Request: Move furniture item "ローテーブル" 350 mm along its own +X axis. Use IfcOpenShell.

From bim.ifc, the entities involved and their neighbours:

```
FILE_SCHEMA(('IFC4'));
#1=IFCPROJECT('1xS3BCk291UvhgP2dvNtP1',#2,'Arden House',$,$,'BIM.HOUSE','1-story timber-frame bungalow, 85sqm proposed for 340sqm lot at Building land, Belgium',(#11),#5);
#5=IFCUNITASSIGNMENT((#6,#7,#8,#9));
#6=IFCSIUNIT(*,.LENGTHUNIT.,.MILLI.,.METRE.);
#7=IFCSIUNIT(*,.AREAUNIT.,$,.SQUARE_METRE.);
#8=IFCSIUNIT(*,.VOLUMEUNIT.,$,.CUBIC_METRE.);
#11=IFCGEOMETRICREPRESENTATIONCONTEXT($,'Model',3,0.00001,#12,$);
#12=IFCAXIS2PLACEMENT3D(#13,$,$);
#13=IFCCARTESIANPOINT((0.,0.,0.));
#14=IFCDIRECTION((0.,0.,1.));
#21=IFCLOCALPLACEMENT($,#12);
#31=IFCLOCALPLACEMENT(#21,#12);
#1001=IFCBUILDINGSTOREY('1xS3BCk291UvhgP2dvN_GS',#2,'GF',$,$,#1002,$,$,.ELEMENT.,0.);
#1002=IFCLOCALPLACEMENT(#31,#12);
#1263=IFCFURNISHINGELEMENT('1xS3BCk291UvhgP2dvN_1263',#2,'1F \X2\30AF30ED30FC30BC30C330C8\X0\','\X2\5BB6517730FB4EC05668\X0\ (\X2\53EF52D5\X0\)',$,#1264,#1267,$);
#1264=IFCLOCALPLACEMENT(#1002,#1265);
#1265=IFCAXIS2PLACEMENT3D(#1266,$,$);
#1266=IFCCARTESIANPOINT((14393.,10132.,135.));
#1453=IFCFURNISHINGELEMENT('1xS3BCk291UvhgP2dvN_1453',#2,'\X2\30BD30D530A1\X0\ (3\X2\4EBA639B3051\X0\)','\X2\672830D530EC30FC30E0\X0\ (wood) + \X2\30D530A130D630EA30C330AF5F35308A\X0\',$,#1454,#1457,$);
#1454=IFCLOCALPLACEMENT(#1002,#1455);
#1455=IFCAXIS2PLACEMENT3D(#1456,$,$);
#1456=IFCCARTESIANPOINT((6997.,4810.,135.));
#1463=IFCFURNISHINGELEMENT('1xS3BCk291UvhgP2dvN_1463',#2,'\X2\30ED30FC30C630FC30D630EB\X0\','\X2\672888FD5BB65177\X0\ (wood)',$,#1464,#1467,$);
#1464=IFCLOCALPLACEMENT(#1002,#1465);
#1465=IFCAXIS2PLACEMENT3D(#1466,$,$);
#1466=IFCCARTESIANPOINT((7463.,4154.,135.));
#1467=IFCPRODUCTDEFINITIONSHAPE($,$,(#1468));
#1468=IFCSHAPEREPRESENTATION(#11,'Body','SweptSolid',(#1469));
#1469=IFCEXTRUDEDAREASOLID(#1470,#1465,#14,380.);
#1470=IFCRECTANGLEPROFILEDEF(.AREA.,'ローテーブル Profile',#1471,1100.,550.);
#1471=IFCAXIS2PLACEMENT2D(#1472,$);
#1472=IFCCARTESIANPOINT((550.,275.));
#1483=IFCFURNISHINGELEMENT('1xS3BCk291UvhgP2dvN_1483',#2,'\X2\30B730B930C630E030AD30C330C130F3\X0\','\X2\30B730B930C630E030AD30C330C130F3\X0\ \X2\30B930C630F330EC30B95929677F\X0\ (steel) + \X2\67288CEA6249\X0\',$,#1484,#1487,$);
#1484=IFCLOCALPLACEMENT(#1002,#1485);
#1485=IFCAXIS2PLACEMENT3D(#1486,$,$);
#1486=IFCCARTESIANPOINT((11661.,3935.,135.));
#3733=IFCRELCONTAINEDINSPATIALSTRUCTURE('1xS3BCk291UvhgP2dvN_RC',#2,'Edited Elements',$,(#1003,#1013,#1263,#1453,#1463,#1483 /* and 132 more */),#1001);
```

```python
import ifcopenshell
import ifcopenshell.api.geometry
import ifcopenshell.util.placement
import ifcopenshell.util.unit

model = ifcopenshell.open("bim.ifc")
unit_scale = ifcopenshell.util.unit.calculate_unit_scale(model)

item = model.by_id(1463)
matrix = ifcopenshell.util.placement.get_local_placement(item.ObjectPlacement)
matrix[:3, 3] += matrix[:3, 0] * 0.35 / unit_scale
ifcopenshell.api.geometry.edit_object_placement(model, product=item, matrix=matrix, is_si=False)

print(ifcopenshell.util.placement.get_local_placement(item.ObjectPlacement).round(3) + 0.0)

model.write("bim_rev.ifc")
```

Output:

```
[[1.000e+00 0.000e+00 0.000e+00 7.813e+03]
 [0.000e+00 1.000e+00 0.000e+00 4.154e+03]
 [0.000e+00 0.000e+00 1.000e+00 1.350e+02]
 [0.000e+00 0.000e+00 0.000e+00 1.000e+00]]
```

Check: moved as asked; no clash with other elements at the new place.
